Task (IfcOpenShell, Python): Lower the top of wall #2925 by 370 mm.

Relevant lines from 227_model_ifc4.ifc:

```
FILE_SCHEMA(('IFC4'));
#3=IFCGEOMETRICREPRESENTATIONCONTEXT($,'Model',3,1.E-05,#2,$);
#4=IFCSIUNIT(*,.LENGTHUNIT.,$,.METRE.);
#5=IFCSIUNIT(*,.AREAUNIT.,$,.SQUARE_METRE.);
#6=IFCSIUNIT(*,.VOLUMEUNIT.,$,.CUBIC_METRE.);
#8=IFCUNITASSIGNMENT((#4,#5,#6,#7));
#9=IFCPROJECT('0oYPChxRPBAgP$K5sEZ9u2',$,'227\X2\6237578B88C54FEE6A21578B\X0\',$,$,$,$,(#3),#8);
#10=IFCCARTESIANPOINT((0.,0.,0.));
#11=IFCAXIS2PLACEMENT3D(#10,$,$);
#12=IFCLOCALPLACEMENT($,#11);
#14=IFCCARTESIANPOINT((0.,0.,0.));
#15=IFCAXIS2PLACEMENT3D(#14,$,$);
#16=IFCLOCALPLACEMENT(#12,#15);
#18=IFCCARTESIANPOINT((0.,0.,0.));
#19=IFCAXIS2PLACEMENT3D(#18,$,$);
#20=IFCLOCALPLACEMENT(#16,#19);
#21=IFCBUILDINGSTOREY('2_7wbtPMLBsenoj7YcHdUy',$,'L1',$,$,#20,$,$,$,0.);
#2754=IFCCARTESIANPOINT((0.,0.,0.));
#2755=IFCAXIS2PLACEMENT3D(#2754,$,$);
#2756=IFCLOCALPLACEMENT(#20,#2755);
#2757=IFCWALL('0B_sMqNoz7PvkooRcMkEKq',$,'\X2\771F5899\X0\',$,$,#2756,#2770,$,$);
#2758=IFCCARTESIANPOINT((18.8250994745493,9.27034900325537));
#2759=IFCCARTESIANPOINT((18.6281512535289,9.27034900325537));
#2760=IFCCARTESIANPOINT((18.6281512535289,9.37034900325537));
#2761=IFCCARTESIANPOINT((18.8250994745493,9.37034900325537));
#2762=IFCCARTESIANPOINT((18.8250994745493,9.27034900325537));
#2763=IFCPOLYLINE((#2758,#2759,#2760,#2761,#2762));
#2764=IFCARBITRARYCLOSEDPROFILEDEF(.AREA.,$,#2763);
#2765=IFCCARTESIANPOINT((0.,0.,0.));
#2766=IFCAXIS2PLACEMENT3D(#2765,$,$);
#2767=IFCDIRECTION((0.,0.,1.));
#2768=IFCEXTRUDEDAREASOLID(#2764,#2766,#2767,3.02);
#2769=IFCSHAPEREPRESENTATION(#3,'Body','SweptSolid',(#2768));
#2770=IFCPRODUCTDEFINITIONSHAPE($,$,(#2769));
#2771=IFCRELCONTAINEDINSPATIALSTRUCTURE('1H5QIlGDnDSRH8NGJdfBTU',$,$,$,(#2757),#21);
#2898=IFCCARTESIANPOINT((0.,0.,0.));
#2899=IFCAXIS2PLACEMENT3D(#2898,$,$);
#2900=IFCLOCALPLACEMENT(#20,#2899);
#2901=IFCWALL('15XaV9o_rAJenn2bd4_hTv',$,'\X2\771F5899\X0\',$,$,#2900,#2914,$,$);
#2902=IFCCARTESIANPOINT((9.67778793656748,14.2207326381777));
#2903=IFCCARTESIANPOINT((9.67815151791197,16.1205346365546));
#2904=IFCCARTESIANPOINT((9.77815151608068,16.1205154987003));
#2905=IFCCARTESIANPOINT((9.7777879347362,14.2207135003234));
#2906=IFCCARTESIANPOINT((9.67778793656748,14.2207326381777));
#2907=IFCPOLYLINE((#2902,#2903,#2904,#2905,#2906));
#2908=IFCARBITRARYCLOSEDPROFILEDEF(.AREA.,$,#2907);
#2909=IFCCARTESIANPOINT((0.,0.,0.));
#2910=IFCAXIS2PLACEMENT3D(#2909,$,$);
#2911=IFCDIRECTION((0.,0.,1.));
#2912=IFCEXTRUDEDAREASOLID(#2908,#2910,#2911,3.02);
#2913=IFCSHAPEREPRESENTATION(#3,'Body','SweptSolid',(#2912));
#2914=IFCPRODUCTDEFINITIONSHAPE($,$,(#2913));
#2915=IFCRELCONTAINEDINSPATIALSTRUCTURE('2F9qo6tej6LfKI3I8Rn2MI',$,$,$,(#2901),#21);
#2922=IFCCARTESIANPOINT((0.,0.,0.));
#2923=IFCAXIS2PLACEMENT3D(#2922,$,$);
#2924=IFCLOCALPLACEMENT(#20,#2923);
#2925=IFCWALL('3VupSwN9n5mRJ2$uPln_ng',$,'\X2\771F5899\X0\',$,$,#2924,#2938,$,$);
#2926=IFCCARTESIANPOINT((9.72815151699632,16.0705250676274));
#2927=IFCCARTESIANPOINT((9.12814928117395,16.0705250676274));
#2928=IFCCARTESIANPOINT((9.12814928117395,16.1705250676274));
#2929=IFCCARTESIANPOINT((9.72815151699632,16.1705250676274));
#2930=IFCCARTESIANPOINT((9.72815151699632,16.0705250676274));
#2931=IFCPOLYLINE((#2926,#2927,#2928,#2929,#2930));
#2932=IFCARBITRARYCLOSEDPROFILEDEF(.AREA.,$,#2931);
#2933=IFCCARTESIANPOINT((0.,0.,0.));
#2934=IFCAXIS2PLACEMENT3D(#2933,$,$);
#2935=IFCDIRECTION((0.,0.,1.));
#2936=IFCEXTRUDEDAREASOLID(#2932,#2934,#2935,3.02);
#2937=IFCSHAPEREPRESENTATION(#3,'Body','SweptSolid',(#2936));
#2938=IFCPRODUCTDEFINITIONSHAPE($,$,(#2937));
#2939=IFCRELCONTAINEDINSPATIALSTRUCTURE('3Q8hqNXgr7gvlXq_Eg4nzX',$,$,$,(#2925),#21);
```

```python
import ifcopenshell
import ifcopenshell.geom
import ifcopenshell.util.shape

model = ifcopenshell.open("227_model_ifc4.ifc")
settings = ifcopenshell.geom.settings()


def volume(element):
    """Net volume in cubic metres, openings subtracted."""
    shape = ifcopenshell.geom.create_shape(settings, element)
    return ifcopenshell.util.shape.get_volume(shape.geometry)


wall = model.by_id(2925)
before = volume(wall)

body = next(r for r in wall.Representation.Representations if r.RepresentationIdentifier == "Body")
solid = body.Items[0]
old_height = solid.Depth
solid.Depth -= 0.37
after = volume(wall)

print(f"height {old_height:g} -> {solid.Depth:g}, volume {before:.3f} -> {after:.3f} m3")

model.write("227_model_ifc4_rev.ifc")
```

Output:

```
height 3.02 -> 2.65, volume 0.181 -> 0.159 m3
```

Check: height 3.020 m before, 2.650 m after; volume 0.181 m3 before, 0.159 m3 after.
